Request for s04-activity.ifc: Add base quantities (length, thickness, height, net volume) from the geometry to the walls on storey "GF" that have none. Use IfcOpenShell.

First a look at what the model holds.

```python
import ifcopenshell
import ifcopenshell.util.element
import ifcopenshell.util.unit

model = ifcopenshell.open("s04-activity.ifc")
print(model.schema)
for unit_type in ("LENGTHUNIT", "AREAUNIT", "VOLUMEUNIT"):
    print(unit_type, ifcopenshell.util.unit.calculate_unit_scale(model, unit_type))
storey = next(s for s in model.by_type("IfcBuildingStorey") if s.Name == "GF")
walls = [e for e in ifcopenshell.util.element.get_decomposition(storey) if e.is_a("IfcWall")]
for e in sorted(walls, key=lambda e: e.id()):
    print(e.id(), e.is_a(), e.Name, list(ifcopenshell.util.element.get_psets(e, qtos_only=True)), sep=" | ")
```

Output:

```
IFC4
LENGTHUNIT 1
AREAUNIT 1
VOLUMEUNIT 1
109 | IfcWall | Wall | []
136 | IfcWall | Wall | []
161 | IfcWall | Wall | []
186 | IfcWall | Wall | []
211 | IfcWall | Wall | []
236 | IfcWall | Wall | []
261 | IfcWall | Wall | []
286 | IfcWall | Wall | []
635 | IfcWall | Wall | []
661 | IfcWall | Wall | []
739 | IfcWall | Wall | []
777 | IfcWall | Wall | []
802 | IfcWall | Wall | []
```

```python
import ifcopenshell
import ifcopenshell.api.pset
import ifcopenshell.geom
import ifcopenshell.util.element
import ifcopenshell.util.shape
import ifcopenshell.util.unit

model = ifcopenshell.open("s04-activity.ifc")
unit_scale = ifcopenshell.util.unit.calculate_unit_scale(model)
volume_scale = ifcopenshell.util.unit.calculate_unit_scale(model, "VOLUMEUNIT")
settings = ifcopenshell.geom.settings()

storey = next(s for s in model.by_type("IfcBuildingStorey") if s.Name == "GF")
walls = [e for e in ifcopenshell.util.element.get_decomposition(storey) if e.is_a("IfcWall")]

for e in sorted(walls, key=lambda e: e.id()):
    if ifcopenshell.util.element.get_psets(e, qtos_only=True, should_inherit=False):
        continue
    # Geometry comes back in metres, in the element's own axes.
    shape = ifcopenshell.geom.create_shape(settings, e)
    values = {
        "Length": ifcopenshell.util.shape.get_x(shape.geometry) / unit_scale,
        "Width": ifcopenshell.util.shape.get_y(shape.geometry) / unit_scale,
        "Height": ifcopenshell.util.shape.get_z(shape.geometry) / unit_scale,
        "NetVolume": ifcopenshell.util.shape.get_volume(shape.geometry) / volume_scale,
    }
    qto = ifcopenshell.api.pset.add_qto(model, product=e, name="Qto_WallBaseQuantities")
    ifcopenshell.api.pset.edit_qto(model, qto=qto, properties=values)
    print(e.id(), {k: round(v, 3) for k, v in values.items()})

model.write("s04-activity_rev.ifc")
```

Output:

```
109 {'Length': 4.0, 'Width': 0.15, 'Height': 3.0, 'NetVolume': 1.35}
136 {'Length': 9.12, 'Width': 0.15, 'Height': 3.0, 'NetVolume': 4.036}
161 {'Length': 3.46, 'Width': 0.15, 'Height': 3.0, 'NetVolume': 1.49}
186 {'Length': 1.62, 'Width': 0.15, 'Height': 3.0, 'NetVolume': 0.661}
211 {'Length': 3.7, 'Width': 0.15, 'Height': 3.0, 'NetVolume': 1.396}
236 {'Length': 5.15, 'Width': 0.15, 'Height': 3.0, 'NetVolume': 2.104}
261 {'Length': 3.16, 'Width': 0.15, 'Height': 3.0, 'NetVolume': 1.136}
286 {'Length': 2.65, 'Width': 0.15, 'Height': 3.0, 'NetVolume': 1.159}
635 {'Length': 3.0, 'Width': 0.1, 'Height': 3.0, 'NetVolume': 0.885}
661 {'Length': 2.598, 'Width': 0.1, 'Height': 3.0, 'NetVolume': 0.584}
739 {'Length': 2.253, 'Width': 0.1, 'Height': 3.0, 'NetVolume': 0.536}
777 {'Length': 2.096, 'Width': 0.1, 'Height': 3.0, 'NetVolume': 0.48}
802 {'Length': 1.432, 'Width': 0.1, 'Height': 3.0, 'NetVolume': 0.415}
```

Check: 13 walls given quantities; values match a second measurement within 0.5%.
